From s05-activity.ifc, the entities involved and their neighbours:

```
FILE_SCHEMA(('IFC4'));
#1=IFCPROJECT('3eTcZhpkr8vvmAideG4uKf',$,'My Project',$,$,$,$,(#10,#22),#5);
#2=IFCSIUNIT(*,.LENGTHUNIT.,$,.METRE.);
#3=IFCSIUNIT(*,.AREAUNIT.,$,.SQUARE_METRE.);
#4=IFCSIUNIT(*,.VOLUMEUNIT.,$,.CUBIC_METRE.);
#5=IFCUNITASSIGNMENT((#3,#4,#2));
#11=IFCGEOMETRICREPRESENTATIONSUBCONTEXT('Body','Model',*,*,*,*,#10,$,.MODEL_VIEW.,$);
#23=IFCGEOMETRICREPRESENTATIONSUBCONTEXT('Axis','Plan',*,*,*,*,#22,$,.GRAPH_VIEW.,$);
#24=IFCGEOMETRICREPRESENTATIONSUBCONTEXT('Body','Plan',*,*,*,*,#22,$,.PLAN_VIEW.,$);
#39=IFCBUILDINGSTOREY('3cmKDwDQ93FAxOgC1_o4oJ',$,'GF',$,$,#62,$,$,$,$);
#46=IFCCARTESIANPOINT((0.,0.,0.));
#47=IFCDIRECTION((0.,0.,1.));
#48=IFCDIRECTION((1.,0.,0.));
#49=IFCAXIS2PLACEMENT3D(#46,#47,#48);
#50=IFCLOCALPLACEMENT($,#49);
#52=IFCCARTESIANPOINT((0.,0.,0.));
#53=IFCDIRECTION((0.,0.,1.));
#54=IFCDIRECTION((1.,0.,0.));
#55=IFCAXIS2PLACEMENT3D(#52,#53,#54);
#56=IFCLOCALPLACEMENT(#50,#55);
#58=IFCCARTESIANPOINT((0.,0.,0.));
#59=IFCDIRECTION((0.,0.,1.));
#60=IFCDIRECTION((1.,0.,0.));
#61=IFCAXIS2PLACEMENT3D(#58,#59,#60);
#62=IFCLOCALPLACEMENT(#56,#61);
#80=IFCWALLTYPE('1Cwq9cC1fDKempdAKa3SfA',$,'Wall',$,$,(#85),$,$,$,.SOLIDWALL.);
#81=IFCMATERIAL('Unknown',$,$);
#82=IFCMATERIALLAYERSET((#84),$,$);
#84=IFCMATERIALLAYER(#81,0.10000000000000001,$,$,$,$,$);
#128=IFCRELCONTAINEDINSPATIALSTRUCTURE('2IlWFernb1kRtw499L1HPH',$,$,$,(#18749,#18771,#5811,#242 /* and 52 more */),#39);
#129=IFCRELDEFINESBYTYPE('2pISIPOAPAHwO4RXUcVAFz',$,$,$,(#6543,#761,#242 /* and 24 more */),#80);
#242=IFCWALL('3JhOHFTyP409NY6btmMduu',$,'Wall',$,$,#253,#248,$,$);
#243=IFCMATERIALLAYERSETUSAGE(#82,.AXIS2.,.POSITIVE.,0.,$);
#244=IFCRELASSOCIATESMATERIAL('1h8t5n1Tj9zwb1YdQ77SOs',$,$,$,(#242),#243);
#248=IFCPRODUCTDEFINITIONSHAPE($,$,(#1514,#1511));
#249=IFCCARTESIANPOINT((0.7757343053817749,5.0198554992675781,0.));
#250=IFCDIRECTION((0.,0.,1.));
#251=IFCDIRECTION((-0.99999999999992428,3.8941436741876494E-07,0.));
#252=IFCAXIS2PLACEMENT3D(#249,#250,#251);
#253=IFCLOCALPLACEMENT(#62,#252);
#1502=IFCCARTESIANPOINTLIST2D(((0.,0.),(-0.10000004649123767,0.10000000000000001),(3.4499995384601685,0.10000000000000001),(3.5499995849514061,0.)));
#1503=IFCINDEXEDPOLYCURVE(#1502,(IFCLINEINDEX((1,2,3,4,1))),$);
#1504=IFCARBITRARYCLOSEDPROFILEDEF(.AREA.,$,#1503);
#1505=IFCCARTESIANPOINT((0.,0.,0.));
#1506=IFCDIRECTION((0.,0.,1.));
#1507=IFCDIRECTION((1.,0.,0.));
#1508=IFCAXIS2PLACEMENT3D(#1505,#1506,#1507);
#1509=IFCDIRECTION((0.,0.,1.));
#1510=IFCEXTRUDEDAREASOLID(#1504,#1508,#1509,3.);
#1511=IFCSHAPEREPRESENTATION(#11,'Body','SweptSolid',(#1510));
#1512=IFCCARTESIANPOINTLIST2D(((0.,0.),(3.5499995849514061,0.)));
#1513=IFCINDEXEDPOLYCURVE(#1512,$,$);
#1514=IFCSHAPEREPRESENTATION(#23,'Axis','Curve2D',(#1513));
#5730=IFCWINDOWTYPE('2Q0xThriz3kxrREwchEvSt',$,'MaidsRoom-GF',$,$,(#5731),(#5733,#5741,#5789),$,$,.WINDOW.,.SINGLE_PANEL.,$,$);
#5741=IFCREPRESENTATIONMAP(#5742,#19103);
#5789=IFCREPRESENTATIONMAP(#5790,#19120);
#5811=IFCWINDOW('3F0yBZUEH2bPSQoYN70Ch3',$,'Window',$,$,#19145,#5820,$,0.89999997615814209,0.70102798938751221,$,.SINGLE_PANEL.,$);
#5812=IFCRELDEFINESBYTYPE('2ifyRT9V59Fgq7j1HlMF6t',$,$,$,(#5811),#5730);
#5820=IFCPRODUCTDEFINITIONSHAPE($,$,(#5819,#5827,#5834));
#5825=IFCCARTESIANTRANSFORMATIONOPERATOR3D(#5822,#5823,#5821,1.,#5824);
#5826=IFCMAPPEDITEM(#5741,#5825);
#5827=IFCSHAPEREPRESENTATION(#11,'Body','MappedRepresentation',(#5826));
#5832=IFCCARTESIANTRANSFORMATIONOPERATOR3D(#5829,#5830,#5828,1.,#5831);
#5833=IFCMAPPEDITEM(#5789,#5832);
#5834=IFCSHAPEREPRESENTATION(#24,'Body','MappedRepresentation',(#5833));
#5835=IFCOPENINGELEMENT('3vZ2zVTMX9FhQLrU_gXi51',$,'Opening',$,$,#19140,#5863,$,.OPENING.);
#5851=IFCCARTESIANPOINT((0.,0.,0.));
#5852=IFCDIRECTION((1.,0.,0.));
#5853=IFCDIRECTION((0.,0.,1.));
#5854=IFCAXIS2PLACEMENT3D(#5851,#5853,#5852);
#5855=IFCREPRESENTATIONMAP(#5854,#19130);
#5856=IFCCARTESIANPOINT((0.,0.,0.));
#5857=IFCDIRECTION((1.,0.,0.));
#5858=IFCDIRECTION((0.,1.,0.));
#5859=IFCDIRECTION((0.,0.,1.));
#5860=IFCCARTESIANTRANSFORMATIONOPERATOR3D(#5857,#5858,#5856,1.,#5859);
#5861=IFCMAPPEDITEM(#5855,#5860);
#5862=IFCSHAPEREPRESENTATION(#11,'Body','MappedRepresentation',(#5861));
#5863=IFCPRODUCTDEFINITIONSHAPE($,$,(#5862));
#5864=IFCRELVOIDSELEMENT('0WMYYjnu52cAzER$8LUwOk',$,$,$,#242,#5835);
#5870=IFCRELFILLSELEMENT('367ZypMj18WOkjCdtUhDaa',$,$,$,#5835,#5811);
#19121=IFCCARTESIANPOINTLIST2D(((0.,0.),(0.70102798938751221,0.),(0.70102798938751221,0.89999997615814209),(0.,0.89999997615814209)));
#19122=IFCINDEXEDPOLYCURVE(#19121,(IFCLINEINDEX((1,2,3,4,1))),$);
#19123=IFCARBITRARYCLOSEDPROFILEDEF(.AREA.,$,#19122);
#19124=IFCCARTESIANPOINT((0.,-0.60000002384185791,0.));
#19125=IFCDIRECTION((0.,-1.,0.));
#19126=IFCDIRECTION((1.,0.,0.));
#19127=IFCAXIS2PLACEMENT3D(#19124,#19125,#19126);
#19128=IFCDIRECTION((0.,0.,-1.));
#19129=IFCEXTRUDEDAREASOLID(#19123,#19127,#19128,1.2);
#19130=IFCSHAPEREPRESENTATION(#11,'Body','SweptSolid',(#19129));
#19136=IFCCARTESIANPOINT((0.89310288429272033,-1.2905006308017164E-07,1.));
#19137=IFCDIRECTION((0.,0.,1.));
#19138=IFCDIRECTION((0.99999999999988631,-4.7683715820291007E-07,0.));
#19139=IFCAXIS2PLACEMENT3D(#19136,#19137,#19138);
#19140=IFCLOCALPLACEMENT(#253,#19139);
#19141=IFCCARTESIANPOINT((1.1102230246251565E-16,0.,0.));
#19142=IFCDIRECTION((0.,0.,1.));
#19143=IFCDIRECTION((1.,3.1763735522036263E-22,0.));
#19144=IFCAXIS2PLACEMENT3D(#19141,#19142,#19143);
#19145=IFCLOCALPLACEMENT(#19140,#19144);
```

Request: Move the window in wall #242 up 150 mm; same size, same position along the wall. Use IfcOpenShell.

```python
import numpy as np
import ifcopenshell
import ifcopenshell.api.geometry
import ifcopenshell.util.placement
import ifcopenshell.util.unit

model = ifcopenshell.open("s05-activity.ifc")
unit_scale = ifcopenshell.util.unit.calculate_unit_scale(model)

window = model.by_guid("3F0yBZUEH2bPSQoYN70Ch3")
opening = window.FillsVoids[0].RelatingOpeningElement
dz = 0.15 / unit_scale

shift = np.array([0.0, 0.0, dz])
# The window is placed relative to its opening, so it follows when the opening moves.
matrix = ifcopenshell.util.placement.get_local_placement(opening.ObjectPlacement)
matrix[:3, 3] += shift
ifcopenshell.api.geometry.edit_object_placement(
    model, product=opening, matrix=matrix, is_si=False, should_transform_children=True
)

print(f"moved by {dz * unit_scale:+.3f} m")

model.write("s05-activity-out.ifc")
```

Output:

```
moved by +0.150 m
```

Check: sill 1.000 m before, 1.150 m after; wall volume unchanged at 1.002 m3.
